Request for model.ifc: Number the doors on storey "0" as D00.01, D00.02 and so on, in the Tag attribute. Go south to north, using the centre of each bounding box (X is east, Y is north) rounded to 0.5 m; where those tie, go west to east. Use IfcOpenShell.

First a look at what the model holds.

```python
import ifcopenshell
import ifcopenshell.util.element
import ifcopenshell.util.placement

model = ifcopenshell.open("model.ifc")
print(model.schema)
storey = next(s for s in model.by_type("IfcBuildingStorey") if s.Name == "0")
doors = [e for e in ifcopenshell.util.element.get_decomposition(storey) if e.is_a("IfcDoor")]
for e in sorted(doors, key=lambda e: e.id()):
    origin = ifcopenshell.util.placement.get_local_placement(e.ObjectPlacement)[:3, 3]
    print(e.id(), e.Tag, e.Name, origin.round(2) + 0.0, sep=" | ")
```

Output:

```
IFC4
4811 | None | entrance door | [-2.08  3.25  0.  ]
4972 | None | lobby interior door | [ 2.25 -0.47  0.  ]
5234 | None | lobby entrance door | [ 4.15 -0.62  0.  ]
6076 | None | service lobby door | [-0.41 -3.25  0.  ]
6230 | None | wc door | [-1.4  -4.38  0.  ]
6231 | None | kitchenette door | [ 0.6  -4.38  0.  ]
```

```python
import ifcopenshell
import ifcopenshell.geom
import ifcopenshell.util.element
import ifcopenshell.util.shape

model = ifcopenshell.open("model.ifc")
settings = ifcopenshell.geom.settings()
settings.set("use-world-coords", True)


def centre(element):
    shape = ifcopenshell.geom.create_shape(settings, element)
    return ifcopenshell.util.shape.get_bbox_centroid(shape.geometry)


storey = next(s for s in model.by_type("IfcBuildingStorey") if s.Name == "0")
doors = [e for e in ifcopenshell.util.element.get_decomposition(storey) if e.is_a("IfcDoor")]

# Insertion points can sit at a corner or the storey origin, so sort by the geometry (in metres).
centres = {e: centre(e) for e in doors}
doors.sort(key=lambda e: (round(centres[e][1] / 0.5), centres[e][0]))

for i, e in enumerate(doors, start=1):
    number = f"D00.{i:02d}"
    e.Tag = number
    print(e.id(), number)

model.write("model_edited.ifc")
```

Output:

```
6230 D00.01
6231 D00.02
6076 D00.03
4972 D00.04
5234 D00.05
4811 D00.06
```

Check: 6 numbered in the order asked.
